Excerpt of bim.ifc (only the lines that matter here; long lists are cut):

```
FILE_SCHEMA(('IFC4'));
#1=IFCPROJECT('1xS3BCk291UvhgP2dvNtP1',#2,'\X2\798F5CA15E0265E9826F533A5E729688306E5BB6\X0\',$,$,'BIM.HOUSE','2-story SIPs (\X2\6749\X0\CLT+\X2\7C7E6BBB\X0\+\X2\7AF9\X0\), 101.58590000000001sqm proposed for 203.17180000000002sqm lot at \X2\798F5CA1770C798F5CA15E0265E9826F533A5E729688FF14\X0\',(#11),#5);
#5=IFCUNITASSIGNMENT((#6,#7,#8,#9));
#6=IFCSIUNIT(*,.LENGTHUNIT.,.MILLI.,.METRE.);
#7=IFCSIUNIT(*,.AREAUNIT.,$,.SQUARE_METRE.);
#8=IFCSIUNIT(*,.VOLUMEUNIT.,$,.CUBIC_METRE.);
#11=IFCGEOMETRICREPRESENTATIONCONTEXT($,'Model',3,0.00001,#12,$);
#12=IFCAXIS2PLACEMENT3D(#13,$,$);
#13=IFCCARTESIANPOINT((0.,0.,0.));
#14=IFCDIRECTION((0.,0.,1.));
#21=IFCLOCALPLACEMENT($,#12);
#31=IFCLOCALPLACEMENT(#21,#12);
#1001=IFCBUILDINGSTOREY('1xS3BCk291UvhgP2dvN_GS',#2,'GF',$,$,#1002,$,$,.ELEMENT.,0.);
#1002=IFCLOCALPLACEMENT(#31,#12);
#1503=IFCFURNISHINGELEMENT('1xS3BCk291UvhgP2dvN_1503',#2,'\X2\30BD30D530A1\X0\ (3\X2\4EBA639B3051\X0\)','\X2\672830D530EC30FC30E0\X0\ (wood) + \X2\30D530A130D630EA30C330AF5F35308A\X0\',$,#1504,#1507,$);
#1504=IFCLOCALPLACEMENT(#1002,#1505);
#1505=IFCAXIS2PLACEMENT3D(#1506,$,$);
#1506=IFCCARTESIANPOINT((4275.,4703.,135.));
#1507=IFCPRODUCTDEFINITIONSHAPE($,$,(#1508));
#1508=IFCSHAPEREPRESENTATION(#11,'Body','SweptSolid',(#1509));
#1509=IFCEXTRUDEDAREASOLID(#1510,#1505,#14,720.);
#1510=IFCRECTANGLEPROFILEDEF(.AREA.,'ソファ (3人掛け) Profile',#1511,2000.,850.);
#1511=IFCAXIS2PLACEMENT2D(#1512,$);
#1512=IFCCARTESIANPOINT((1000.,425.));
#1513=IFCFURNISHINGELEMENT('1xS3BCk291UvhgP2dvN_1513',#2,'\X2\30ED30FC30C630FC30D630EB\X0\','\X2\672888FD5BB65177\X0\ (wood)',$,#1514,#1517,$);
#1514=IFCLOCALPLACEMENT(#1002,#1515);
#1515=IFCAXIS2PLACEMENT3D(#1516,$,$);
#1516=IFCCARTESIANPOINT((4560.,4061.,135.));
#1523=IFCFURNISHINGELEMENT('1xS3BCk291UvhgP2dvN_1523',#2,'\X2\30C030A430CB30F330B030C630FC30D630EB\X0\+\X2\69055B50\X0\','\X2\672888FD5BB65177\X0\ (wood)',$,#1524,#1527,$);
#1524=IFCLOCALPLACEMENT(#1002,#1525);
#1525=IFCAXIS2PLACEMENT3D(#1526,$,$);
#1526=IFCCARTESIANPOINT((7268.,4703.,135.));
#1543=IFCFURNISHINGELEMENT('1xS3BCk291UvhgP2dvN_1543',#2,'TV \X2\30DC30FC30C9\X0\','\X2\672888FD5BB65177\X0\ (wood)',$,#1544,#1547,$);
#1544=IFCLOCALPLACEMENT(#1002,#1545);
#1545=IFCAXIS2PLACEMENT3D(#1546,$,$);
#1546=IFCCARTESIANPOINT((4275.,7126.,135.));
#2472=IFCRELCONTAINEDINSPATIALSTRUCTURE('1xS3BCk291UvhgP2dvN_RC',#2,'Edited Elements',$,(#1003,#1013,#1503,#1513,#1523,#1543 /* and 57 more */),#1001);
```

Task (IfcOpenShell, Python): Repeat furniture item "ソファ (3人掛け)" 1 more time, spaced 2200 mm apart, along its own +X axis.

```python
import ifcopenshell
import ifcopenshell.api.geometry
import ifcopenshell.api.root
import ifcopenshell.util.element
import ifcopenshell.util.placement

model = ifcopenshell.open("bim.ifc")


def reuse_history(source, copy):
    """copy_class also copies each property set's owner history, people and application; keep the originals."""
    for rel in copy.IsDefinedBy:
        if rel.is_a("IfcRelDefinesByProperties") and (history := rel.RelatingPropertyDefinition.OwnerHistory):
            rel.RelatingPropertyDefinition.OwnerHistory = source.OwnerHistory
            ifcopenshell.util.element.remove_deep2(model, history)


source = model.by_guid("1xS3BCk291UvhgP2dvN_1503")
base = ifcopenshell.util.placement.get_local_placement(source.ObjectPlacement)
step = base[:3, 0] * 2200.0

for i in range(1, 2):
    copy = ifcopenshell.api.root.copy_class(model, product=source)
    copy.Representation = ifcopenshell.util.element.copy_deep(
        model, source.Representation, exclude=["IfcGeometricRepresentationContext", "IfcRepresentationMap"]
    )
    reuse_history(source, copy)
    matrix = base.copy()
    matrix[:3, 3] += i * step
    print("added at", matrix[:3, 3].round(3) + 0.0)
    ifcopenshell.api.geometry.edit_object_placement(model, product=copy, matrix=matrix, is_si=False)

model.write("bim_edited.ifc")
```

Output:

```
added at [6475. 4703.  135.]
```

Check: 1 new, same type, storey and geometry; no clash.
